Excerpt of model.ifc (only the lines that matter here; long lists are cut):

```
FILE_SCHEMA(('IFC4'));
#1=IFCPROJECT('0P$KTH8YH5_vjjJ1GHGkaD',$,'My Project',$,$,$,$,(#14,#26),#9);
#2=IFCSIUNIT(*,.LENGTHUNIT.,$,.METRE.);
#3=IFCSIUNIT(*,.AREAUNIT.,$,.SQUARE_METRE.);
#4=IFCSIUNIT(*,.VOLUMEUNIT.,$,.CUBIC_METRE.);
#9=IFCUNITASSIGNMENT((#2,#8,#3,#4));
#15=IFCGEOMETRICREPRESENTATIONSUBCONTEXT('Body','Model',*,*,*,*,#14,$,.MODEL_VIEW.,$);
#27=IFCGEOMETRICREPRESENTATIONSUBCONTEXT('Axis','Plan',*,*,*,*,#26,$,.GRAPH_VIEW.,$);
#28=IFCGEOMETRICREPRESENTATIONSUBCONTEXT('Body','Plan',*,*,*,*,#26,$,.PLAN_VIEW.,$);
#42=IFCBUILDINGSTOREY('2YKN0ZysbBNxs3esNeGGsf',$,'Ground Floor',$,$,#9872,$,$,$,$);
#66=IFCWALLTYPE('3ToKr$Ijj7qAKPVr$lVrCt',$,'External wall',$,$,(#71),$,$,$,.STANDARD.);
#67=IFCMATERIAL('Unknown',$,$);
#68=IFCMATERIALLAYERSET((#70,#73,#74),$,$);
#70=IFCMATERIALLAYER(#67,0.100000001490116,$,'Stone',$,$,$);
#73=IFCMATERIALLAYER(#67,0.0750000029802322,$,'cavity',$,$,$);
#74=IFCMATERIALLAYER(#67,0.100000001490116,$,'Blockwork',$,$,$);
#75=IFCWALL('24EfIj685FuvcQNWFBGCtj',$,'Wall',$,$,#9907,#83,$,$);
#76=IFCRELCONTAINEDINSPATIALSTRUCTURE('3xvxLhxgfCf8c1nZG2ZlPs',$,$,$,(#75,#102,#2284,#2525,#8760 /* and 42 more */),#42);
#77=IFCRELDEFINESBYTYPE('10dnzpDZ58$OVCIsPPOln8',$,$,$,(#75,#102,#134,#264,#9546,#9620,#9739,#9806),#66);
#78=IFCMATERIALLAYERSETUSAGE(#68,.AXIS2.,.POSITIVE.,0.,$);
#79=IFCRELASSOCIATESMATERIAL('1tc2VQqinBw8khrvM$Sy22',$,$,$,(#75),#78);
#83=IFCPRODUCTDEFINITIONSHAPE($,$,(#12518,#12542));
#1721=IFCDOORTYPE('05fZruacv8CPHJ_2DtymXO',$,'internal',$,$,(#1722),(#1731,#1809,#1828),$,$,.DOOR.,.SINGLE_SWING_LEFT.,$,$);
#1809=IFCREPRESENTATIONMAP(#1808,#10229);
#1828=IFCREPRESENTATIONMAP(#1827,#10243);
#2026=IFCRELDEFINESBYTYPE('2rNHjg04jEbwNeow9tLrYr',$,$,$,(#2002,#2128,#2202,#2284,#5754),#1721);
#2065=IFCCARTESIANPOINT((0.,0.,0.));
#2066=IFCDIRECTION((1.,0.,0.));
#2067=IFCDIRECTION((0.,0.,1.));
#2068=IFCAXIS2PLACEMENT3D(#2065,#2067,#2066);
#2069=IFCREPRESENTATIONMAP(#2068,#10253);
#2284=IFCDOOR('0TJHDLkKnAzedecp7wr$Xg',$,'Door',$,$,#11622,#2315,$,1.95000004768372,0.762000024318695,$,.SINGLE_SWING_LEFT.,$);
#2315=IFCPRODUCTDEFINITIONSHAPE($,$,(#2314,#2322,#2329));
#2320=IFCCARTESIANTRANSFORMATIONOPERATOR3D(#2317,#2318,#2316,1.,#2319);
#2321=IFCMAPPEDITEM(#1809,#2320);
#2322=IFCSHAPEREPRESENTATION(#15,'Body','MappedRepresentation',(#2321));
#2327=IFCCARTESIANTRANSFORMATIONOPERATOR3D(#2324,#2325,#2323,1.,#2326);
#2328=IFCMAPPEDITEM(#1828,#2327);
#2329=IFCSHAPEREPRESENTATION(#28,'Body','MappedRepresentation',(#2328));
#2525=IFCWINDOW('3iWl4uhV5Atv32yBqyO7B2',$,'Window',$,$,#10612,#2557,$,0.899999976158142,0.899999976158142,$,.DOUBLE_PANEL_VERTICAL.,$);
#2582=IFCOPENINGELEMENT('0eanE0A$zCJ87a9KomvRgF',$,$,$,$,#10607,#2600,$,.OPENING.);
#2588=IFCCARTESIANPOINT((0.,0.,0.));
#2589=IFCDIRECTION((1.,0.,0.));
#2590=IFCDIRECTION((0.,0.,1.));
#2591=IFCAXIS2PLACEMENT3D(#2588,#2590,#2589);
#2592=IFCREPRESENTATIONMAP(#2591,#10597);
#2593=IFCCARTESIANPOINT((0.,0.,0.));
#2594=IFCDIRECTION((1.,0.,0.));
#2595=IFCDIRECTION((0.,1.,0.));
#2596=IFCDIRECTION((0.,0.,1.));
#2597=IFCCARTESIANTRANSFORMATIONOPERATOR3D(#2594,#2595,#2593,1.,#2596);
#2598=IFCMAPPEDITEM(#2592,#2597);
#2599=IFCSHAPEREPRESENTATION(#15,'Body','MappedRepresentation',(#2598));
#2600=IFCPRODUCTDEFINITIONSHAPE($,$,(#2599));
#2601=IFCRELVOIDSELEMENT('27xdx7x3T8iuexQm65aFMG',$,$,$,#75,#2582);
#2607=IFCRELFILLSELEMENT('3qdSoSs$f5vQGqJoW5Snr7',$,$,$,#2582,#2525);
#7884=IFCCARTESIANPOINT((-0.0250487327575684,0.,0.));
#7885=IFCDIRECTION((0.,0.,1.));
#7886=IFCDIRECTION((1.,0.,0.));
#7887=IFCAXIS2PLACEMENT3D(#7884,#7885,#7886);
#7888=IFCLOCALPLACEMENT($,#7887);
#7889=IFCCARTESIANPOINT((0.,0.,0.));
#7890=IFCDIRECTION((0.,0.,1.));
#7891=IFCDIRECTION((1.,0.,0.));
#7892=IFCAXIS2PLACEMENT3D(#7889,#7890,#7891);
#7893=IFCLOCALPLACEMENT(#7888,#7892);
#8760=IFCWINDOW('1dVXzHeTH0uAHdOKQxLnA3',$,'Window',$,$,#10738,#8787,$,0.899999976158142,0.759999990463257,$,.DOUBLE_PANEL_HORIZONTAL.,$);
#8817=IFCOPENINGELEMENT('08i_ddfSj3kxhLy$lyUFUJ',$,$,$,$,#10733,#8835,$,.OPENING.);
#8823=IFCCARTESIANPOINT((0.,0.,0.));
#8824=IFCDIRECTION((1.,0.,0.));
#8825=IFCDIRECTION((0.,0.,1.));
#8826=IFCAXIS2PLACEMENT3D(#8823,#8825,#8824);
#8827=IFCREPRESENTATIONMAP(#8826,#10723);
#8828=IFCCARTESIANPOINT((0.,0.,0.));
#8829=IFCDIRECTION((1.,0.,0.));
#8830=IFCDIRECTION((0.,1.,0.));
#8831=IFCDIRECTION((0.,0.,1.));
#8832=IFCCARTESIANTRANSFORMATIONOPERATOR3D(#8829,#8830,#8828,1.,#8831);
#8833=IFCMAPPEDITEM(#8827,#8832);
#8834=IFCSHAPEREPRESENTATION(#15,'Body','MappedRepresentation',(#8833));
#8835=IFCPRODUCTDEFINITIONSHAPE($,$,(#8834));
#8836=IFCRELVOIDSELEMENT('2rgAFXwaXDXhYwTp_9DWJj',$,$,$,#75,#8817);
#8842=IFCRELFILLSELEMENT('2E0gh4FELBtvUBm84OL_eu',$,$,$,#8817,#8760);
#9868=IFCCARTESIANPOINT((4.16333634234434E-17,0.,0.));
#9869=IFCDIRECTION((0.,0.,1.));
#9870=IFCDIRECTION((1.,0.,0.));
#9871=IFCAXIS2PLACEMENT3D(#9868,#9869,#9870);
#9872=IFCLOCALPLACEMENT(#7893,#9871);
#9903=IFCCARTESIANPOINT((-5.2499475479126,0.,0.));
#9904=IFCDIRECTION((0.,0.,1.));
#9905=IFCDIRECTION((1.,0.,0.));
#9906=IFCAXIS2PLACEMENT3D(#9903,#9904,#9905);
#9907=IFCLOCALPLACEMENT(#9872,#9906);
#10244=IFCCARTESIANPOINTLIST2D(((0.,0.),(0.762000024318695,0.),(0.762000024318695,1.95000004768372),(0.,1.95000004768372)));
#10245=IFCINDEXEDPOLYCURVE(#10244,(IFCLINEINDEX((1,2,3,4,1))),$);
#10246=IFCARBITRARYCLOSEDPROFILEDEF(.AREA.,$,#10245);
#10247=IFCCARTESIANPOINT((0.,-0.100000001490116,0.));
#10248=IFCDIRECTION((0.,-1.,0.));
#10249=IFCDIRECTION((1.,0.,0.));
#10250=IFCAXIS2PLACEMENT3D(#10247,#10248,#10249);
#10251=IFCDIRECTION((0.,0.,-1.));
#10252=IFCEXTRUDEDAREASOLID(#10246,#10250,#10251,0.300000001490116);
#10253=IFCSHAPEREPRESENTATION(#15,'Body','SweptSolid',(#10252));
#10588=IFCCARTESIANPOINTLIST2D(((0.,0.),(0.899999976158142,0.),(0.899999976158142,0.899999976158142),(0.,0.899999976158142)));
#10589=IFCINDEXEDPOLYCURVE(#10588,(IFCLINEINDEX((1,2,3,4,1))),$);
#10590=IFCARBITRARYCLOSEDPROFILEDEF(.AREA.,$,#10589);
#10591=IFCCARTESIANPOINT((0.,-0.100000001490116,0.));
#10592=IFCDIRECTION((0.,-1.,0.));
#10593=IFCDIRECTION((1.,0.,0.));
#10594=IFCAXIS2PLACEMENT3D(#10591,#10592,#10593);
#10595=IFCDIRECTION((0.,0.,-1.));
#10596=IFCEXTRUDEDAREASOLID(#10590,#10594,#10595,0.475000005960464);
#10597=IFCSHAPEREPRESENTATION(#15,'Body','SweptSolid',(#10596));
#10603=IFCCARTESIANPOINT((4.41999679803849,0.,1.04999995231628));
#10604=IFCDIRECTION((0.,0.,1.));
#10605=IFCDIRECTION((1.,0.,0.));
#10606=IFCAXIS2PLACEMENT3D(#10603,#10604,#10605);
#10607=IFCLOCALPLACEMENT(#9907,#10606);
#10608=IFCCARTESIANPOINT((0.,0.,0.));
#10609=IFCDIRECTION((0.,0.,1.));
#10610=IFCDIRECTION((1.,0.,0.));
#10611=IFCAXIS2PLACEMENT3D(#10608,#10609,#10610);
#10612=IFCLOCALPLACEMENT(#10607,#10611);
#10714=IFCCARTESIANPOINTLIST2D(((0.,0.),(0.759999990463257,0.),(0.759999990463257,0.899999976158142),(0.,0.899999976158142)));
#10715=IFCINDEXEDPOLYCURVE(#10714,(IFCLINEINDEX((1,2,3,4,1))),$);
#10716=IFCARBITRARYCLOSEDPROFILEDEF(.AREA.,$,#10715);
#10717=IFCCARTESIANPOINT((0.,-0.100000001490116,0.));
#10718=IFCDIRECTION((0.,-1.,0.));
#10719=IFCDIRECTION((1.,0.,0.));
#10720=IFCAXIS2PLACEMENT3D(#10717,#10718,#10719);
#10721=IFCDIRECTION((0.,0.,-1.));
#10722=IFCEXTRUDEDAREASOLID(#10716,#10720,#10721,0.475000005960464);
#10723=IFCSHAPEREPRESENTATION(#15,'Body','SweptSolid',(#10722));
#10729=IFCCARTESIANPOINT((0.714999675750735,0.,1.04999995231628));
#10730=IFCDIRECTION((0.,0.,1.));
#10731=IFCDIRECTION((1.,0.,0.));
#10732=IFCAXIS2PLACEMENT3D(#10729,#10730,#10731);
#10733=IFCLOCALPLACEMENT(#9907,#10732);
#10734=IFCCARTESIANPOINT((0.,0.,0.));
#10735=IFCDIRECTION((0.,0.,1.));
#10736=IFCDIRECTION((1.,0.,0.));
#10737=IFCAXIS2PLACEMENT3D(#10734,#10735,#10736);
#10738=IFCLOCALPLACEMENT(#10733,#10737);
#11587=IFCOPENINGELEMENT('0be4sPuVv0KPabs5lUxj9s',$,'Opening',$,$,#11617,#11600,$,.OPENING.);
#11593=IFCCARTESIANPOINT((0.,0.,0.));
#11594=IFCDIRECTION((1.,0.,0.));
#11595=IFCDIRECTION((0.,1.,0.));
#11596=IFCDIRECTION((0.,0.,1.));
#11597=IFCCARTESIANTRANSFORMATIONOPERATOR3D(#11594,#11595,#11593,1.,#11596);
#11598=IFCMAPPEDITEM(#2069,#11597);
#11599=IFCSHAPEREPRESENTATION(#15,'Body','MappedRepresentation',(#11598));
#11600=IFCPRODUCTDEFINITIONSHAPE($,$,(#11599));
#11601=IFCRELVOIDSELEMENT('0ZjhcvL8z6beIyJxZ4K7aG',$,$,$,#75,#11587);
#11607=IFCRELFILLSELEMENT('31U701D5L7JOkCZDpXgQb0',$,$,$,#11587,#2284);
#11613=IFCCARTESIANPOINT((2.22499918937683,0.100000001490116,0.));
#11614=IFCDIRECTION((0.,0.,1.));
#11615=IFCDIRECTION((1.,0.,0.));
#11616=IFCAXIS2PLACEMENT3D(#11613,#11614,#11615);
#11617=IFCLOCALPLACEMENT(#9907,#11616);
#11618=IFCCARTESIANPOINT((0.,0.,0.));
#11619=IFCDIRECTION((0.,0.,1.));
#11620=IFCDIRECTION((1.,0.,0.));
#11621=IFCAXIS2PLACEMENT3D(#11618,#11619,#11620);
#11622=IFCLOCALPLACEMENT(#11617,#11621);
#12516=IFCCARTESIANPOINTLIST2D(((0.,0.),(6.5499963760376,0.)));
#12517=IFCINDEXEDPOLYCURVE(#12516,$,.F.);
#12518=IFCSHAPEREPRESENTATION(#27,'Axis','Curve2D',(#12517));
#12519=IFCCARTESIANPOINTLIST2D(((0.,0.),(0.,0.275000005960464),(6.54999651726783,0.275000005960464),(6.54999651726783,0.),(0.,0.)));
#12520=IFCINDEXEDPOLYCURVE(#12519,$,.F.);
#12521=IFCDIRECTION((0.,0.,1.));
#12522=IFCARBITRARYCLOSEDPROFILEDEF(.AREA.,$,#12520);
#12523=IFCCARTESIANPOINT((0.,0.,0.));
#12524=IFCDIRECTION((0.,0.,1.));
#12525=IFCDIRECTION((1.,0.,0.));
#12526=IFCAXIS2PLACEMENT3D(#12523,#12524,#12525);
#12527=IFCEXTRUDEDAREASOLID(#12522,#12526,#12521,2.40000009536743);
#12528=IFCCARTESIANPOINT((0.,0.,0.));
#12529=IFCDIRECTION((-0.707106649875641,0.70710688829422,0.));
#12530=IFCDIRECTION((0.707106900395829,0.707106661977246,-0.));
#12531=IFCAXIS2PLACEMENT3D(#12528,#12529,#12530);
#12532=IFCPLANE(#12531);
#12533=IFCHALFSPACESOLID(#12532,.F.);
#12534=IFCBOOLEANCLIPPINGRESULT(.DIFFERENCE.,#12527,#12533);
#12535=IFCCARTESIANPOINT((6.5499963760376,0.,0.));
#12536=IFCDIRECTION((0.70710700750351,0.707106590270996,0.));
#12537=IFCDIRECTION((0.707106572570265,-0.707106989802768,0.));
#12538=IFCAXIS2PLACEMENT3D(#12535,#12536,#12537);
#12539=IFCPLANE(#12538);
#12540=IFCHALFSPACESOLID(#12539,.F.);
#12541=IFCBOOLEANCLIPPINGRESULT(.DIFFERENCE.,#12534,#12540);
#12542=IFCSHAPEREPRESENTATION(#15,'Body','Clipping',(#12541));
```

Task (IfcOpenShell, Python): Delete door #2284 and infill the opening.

```python
import ifcopenshell
import ifcopenshell.api.feature
import ifcopenshell.api.root
import ifcopenshell.geom
import ifcopenshell.util.shape

model = ifcopenshell.open("model.ifc")
settings = ifcopenshell.geom.settings()


def volume(element):
    """Net volume in cubic metres, openings subtracted."""
    shape = ifcopenshell.geom.create_shape(settings, element)
    return ifcopenshell.util.shape.get_volume(shape.geometry)


door = model.by_guid("0TJHDLkKnAzedecp7wr$Xg")
opening = door.FillsVoids[0].RelatingOpeningElement
wall = opening.VoidsElements[0].RelatingBuildingElement
before = volume(wall)

ifcopenshell.api.root.remove_product(model, product=door)
ifcopenshell.api.feature.remove_feature(model, feature=opening)

after = volume(wall)

print(f"wall volume {before:.3f} -> {after:.3f} m3")

model.write("model_edited.ifc")
```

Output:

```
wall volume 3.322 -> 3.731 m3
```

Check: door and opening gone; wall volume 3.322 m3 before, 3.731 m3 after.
